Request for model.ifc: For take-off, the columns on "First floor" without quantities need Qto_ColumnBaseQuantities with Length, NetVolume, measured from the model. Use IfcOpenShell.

First a look at what the model holds.

```python
import ifcopenshell
import ifcopenshell.util.element
import ifcopenshell.util.unit

model = ifcopenshell.open("model.ifc")
print(model.schema)
for unit_type in ("LENGTHUNIT", "AREAUNIT", "VOLUMEUNIT"):
    print(unit_type, ifcopenshell.util.unit.calculate_unit_scale(model, unit_type))
storey = next(s for s in model.by_type("IfcBuildingStorey") if s.Name == "First floor")
columns = [e for e in ifcopenshell.util.element.get_decomposition(storey) if e.is_a("IfcColumn")]
for e in sorted(columns, key=lambda e: e.id()):
    print(e.id(), e.is_a(), e.Name, list(ifcopenshell.util.element.get_psets(e, qtos_only=True)), sep=" | ")
```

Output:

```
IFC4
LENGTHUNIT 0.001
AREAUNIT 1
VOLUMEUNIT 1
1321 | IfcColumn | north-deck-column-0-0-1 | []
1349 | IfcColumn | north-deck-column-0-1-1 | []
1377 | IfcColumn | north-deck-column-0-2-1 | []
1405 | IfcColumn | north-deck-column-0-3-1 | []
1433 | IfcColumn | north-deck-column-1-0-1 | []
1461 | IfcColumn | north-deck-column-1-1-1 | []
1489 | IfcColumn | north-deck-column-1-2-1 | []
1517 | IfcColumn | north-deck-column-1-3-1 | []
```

```python
import ifcopenshell
import ifcopenshell.api.pset
import ifcopenshell.geom
import ifcopenshell.util.element
import ifcopenshell.util.shape
import ifcopenshell.util.unit

model = ifcopenshell.open("model.ifc")
unit_scale = ifcopenshell.util.unit.calculate_unit_scale(model)
volume_scale = ifcopenshell.util.unit.calculate_unit_scale(model, "VOLUMEUNIT")
settings = ifcopenshell.geom.settings()

storey = next(s for s in model.by_type("IfcBuildingStorey") if s.Name == "First floor")
columns = [e for e in ifcopenshell.util.element.get_decomposition(storey) if e.is_a("IfcColumn")]

for e in sorted(columns, key=lambda e: e.id()):
    if ifcopenshell.util.element.get_psets(e, qtos_only=True, should_inherit=False):
        continue
    # Geometry comes back in metres, in the element's own axes.
    shape = ifcopenshell.geom.create_shape(settings, e)
    values = {
        "Length": ifcopenshell.util.shape.get_z(shape.geometry) / unit_scale,
        "NetVolume": ifcopenshell.util.shape.get_volume(shape.geometry) / volume_scale,
    }
    qto = ifcopenshell.api.pset.add_qto(model, product=e, name="Qto_ColumnBaseQuantities")
    ifcopenshell.api.pset.edit_qto(model, qto=qto, properties=values)
    print(e.id(), {k: round(v, 3) for k, v in values.items()})

model.write("model_updated.ifc")
```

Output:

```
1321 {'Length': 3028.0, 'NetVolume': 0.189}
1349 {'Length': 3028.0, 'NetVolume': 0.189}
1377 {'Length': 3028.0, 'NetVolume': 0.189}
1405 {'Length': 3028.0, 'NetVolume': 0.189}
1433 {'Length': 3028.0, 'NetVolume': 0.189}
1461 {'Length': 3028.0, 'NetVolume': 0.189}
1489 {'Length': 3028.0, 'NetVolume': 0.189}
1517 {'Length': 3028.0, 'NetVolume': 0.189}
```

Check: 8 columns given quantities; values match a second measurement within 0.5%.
